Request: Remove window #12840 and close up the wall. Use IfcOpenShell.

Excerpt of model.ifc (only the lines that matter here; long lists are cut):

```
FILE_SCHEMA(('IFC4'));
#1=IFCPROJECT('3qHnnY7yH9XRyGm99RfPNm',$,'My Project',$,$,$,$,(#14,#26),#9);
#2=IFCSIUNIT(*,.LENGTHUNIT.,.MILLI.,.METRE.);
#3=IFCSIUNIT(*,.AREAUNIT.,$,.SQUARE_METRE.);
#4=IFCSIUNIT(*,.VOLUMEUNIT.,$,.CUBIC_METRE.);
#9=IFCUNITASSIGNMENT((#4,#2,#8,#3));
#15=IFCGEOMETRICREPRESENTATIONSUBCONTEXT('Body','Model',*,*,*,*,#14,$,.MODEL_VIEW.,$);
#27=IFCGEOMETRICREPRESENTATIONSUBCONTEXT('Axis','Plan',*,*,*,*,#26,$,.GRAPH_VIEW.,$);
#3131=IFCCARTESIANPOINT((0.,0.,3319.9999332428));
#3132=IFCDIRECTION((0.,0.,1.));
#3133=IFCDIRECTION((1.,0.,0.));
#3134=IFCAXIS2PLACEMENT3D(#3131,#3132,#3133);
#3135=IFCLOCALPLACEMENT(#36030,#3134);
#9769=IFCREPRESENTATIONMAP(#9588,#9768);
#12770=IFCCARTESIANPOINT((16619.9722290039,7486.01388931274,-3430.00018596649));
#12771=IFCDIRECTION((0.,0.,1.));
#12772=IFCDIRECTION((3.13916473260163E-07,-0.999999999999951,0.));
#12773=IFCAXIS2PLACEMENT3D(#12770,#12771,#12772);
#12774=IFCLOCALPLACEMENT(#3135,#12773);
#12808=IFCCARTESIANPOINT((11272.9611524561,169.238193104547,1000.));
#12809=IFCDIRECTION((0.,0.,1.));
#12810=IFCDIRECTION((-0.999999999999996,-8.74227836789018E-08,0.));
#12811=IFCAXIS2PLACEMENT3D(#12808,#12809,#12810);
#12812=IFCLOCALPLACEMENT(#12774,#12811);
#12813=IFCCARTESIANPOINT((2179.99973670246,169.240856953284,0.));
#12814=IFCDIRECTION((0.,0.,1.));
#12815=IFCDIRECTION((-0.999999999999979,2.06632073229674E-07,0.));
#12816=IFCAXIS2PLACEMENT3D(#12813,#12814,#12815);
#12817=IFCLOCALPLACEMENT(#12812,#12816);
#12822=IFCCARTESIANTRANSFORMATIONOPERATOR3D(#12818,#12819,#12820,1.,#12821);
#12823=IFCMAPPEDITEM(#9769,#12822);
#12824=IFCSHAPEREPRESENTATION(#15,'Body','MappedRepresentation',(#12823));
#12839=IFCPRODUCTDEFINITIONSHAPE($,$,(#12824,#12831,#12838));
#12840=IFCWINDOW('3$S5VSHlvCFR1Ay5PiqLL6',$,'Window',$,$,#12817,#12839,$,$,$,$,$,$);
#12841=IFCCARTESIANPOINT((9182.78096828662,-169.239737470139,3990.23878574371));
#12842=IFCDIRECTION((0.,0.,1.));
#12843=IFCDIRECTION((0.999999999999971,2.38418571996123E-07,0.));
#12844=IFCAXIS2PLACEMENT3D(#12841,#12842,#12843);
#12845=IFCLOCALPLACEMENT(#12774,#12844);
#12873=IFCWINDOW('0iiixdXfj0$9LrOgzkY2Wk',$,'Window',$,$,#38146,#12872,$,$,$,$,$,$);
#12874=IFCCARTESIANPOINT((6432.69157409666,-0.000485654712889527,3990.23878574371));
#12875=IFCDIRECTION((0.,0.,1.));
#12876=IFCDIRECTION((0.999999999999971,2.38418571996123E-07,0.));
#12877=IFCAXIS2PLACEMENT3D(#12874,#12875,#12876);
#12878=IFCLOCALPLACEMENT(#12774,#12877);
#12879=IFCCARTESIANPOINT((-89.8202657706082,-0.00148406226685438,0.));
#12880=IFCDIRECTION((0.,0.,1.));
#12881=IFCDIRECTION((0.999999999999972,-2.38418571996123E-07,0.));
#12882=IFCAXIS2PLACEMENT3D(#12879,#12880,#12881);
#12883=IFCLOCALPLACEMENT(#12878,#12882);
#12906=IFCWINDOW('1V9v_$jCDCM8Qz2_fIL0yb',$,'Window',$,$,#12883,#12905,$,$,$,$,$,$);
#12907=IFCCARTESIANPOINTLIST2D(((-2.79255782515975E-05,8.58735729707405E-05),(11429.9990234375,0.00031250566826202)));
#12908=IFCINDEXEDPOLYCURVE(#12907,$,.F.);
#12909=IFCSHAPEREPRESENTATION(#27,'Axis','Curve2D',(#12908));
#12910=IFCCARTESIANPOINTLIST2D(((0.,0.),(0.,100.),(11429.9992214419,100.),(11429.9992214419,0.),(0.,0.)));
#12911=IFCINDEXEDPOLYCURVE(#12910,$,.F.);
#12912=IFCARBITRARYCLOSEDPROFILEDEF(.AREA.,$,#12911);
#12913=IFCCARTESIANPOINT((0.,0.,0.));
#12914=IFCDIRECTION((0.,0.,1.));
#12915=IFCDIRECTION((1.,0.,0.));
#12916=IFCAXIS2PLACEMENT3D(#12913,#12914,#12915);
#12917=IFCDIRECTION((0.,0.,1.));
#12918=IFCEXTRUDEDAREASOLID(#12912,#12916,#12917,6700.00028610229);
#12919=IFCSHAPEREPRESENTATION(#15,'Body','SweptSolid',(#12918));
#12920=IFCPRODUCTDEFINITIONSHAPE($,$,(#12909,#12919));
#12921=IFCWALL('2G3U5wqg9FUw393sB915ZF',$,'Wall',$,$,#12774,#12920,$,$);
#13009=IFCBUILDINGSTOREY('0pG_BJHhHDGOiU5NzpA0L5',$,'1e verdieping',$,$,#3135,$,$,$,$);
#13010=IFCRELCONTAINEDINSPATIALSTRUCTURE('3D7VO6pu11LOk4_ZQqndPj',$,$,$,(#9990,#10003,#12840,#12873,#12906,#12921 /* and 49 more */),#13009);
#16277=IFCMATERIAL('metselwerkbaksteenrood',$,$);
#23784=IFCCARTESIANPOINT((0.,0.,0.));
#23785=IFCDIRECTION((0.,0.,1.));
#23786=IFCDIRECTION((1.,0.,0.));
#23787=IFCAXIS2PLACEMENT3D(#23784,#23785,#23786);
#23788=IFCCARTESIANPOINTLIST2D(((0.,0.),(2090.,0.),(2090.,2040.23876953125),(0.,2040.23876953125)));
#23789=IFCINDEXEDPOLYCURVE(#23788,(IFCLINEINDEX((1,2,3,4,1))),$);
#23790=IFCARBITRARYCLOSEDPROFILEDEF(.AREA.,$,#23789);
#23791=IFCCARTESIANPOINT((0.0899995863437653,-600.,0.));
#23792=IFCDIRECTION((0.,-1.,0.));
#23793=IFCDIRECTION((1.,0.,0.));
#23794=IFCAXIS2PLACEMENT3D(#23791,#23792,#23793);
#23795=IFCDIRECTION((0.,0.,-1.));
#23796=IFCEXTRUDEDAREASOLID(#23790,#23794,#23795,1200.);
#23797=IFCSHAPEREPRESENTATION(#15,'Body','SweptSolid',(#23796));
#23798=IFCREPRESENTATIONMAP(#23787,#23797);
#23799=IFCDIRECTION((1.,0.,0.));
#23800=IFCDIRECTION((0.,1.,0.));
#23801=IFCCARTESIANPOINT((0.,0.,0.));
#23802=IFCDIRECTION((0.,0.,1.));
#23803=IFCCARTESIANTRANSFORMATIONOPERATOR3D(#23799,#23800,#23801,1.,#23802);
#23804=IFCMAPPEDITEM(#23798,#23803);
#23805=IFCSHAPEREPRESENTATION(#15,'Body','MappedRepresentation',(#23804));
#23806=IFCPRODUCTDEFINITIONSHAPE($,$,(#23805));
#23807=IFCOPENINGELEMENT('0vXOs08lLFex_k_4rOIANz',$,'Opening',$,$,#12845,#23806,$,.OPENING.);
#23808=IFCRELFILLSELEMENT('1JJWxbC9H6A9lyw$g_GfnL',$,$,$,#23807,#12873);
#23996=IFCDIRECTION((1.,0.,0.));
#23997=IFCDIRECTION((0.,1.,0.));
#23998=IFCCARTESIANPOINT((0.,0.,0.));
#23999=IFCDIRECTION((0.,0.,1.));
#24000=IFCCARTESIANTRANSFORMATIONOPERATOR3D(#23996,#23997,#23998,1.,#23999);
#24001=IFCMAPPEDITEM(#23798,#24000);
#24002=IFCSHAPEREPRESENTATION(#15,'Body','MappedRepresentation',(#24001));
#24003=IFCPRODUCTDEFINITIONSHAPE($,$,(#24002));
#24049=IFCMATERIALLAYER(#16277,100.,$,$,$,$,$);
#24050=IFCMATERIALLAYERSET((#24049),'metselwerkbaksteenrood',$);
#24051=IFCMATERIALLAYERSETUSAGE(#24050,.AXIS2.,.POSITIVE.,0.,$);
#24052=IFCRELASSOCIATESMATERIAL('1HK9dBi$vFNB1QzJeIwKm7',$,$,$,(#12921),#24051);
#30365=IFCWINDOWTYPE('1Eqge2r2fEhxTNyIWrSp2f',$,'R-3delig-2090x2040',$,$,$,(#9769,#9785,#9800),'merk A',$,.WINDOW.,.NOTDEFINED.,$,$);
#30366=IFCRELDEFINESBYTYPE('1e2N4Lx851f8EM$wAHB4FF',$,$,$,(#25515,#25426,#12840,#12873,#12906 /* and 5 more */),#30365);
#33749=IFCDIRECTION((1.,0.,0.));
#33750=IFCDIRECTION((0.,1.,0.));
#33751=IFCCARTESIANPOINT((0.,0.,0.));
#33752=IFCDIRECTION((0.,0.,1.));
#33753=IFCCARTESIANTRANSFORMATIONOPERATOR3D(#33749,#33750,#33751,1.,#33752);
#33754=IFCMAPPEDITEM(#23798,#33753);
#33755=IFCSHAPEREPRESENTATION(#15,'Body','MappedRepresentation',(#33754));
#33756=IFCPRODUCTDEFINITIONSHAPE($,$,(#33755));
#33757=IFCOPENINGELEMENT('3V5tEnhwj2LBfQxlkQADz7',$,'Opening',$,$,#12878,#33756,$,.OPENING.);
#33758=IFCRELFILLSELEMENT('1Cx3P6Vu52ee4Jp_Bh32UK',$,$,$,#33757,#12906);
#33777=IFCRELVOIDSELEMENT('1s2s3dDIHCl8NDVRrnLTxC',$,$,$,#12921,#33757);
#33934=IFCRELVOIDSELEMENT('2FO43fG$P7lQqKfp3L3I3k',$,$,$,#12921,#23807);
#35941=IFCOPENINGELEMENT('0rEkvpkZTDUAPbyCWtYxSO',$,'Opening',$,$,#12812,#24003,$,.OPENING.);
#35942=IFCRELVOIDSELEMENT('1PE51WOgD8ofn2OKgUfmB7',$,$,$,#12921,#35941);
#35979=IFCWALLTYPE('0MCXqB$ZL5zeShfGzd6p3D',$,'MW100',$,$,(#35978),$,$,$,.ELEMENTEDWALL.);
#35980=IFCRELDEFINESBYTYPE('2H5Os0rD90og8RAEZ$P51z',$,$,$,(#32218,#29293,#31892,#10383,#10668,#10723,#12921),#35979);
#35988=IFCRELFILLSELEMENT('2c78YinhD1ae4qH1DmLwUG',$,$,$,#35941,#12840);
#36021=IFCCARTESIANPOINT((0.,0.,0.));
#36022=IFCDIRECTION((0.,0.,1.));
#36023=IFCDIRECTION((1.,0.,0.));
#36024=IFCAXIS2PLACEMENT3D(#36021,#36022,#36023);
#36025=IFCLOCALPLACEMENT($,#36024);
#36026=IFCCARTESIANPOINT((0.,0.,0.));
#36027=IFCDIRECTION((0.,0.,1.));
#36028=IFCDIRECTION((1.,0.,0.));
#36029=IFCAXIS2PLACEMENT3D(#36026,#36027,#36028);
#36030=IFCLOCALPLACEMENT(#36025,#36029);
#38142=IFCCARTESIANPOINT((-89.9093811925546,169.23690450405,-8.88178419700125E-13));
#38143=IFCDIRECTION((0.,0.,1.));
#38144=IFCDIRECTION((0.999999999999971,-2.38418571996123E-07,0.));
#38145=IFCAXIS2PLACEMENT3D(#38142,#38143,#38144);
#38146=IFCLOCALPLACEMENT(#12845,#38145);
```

```python
import ifcopenshell
import ifcopenshell.api.feature
import ifcopenshell.api.root
import ifcopenshell.geom
import ifcopenshell.util.shape

model = ifcopenshell.open("model.ifc")
settings = ifcopenshell.geom.settings()


def volume(element):
    """Net volume in cubic metres, openings subtracted."""
    shape = ifcopenshell.geom.create_shape(settings, element)
    return ifcopenshell.util.shape.get_volume(shape.geometry)


window = model.by_guid("3$S5VSHlvCFR1Ay5PiqLL6")
opening = window.FillsVoids[0].RelatingOpeningElement
wall = opening.VoidsElements[0].RelatingBuildingElement
before = volume(wall)

ifcopenshell.api.root.remove_product(model, product=window)
ifcopenshell.api.feature.remove_feature(model, feature=opening)

after = volume(wall)

print(f"wall volume {before:.3f} -> {after:.3f} m3")

model.write("model_updated.ifc")
```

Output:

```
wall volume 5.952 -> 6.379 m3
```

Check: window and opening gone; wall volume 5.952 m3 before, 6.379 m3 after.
